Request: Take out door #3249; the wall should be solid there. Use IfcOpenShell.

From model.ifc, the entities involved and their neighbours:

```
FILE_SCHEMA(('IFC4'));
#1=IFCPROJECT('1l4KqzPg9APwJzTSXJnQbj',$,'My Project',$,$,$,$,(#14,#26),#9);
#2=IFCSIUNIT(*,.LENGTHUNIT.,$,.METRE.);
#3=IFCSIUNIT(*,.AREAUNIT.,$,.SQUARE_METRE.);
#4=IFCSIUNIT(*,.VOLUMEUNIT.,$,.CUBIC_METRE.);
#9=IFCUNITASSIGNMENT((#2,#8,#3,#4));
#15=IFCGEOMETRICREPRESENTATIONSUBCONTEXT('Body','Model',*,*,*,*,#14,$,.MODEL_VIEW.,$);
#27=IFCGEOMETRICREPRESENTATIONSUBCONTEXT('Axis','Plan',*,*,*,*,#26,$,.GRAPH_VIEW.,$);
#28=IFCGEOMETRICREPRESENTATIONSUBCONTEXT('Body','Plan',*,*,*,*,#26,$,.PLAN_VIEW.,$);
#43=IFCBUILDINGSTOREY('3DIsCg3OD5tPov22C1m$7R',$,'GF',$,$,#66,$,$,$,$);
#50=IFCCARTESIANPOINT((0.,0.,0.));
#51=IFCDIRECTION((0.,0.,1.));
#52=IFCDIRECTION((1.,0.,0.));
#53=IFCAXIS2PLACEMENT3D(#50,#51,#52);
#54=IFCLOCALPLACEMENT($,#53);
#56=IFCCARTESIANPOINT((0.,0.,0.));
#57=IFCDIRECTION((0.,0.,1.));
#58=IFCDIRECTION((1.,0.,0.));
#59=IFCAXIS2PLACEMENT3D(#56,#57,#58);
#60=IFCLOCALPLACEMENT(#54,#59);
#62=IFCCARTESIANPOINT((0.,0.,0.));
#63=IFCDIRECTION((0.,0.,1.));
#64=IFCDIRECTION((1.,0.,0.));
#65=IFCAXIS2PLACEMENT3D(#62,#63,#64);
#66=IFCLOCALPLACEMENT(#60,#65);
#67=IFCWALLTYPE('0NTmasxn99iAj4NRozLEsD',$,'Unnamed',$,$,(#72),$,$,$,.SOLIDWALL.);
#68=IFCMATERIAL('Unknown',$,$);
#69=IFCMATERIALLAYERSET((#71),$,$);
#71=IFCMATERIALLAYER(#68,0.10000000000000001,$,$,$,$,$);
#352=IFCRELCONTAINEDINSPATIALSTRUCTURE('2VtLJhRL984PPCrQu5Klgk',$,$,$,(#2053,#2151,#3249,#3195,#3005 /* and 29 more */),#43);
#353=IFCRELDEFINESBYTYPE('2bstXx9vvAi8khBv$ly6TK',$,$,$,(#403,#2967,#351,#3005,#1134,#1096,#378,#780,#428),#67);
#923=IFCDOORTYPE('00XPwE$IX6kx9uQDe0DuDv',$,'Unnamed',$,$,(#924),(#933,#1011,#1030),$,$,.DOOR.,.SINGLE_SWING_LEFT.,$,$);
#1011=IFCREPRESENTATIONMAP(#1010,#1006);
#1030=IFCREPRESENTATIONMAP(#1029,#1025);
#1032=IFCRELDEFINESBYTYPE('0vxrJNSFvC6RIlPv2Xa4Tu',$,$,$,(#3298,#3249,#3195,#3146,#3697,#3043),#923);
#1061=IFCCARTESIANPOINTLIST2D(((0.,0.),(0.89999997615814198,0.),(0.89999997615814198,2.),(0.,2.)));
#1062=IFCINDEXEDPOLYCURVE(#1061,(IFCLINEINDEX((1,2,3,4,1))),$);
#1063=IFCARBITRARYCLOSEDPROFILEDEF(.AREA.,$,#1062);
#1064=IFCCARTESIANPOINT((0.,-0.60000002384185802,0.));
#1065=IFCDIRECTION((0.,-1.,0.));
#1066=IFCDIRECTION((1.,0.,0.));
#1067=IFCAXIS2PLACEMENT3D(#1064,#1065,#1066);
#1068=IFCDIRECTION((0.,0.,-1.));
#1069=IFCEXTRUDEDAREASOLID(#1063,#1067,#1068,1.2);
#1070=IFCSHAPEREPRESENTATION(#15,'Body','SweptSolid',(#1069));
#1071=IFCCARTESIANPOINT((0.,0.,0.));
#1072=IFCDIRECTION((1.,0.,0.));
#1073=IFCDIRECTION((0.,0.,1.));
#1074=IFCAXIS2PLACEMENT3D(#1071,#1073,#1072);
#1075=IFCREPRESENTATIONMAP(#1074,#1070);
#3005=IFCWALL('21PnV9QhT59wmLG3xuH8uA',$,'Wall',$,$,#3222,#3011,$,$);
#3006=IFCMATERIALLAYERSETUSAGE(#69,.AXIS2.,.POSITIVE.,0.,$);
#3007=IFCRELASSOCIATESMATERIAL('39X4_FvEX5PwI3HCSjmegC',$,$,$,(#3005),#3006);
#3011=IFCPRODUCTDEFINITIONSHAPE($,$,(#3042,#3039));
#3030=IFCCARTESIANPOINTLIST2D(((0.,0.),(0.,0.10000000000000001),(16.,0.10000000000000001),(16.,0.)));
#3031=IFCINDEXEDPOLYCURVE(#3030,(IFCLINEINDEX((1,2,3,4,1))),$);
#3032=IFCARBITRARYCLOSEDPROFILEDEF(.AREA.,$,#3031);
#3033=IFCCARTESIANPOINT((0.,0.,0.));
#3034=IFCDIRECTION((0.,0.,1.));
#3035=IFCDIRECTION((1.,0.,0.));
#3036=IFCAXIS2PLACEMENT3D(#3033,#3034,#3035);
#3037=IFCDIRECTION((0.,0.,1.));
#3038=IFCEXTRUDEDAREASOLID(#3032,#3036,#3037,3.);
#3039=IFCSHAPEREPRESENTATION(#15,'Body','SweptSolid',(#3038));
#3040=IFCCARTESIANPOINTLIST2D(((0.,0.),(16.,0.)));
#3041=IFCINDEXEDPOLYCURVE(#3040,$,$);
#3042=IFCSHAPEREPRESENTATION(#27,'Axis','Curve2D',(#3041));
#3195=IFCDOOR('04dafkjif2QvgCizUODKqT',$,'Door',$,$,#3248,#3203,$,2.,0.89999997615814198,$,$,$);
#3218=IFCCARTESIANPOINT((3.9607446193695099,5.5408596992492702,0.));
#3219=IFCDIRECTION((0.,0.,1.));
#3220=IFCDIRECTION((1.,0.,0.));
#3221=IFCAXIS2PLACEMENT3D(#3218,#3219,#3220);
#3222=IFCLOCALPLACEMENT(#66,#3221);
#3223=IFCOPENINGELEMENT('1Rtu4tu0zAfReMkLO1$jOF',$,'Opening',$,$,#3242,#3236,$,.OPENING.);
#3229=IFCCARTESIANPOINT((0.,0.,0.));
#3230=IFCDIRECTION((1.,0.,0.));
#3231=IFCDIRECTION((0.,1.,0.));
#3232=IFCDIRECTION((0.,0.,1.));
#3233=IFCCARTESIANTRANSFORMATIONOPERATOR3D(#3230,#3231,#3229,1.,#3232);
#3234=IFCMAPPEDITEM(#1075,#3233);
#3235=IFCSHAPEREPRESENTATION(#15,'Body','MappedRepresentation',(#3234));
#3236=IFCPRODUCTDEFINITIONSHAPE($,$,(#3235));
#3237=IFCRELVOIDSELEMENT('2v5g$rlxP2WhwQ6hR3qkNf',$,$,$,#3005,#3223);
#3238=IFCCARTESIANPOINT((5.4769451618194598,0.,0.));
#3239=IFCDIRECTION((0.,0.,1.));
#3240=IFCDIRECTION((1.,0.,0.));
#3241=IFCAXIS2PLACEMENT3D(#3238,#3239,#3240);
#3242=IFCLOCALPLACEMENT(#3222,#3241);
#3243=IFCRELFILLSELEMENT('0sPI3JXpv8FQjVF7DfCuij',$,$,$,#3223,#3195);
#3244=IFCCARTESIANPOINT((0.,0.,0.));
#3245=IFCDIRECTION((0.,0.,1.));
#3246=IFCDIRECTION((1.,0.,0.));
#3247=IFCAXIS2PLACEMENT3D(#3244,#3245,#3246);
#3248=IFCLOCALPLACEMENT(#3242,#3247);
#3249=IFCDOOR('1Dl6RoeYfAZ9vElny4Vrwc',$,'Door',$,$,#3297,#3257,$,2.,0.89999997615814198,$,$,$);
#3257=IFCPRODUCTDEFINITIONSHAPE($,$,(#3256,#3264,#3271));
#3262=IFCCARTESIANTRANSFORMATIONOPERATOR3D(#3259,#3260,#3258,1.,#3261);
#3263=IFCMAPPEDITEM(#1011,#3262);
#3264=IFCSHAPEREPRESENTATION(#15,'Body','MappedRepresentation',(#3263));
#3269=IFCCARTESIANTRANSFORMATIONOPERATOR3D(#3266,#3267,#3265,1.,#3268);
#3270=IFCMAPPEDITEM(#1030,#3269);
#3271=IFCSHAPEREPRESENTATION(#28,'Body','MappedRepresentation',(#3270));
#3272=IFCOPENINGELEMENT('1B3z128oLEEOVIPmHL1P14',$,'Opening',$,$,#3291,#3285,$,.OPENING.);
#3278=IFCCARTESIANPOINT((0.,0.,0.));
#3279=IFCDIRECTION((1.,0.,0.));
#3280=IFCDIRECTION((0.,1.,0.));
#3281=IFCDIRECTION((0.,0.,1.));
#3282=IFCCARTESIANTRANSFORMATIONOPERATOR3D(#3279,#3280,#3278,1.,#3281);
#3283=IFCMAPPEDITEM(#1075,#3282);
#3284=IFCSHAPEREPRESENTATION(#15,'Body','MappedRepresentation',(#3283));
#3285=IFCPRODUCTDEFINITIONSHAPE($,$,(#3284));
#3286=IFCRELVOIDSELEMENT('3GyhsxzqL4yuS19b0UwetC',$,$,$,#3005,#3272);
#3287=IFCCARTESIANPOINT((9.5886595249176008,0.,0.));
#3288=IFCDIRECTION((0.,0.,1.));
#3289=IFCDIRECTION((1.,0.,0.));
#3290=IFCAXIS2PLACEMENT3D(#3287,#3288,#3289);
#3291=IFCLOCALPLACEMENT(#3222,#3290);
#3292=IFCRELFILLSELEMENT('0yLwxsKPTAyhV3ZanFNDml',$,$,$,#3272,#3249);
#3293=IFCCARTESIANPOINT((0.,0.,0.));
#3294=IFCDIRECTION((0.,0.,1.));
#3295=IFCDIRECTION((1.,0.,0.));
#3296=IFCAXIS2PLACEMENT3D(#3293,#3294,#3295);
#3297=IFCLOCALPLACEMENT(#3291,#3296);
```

```python
import ifcopenshell
import ifcopenshell.api.feature
import ifcopenshell.api.root
import ifcopenshell.geom
import ifcopenshell.util.shape

model = ifcopenshell.open("model.ifc")
settings = ifcopenshell.geom.settings()


def volume(element):
    """Net volume in cubic metres, openings subtracted."""
    shape = ifcopenshell.geom.create_shape(settings, element)
    return ifcopenshell.util.shape.get_volume(shape.geometry)


door = model.by_guid("1Dl6RoeYfAZ9vElny4Vrwc")
opening = door.FillsVoids[0].RelatingOpeningElement
wall = opening.VoidsElements[0].RelatingBuildingElement
before = volume(wall)

ifcopenshell.api.root.remove_product(model, product=door)
ifcopenshell.api.feature.remove_feature(model, feature=opening)

after = volume(wall)

print(f"wall volume {before:.3f} -> {after:.3f} m3")

model.write("model_v2.ifc")
```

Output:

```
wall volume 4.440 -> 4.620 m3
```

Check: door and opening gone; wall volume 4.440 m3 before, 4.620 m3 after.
